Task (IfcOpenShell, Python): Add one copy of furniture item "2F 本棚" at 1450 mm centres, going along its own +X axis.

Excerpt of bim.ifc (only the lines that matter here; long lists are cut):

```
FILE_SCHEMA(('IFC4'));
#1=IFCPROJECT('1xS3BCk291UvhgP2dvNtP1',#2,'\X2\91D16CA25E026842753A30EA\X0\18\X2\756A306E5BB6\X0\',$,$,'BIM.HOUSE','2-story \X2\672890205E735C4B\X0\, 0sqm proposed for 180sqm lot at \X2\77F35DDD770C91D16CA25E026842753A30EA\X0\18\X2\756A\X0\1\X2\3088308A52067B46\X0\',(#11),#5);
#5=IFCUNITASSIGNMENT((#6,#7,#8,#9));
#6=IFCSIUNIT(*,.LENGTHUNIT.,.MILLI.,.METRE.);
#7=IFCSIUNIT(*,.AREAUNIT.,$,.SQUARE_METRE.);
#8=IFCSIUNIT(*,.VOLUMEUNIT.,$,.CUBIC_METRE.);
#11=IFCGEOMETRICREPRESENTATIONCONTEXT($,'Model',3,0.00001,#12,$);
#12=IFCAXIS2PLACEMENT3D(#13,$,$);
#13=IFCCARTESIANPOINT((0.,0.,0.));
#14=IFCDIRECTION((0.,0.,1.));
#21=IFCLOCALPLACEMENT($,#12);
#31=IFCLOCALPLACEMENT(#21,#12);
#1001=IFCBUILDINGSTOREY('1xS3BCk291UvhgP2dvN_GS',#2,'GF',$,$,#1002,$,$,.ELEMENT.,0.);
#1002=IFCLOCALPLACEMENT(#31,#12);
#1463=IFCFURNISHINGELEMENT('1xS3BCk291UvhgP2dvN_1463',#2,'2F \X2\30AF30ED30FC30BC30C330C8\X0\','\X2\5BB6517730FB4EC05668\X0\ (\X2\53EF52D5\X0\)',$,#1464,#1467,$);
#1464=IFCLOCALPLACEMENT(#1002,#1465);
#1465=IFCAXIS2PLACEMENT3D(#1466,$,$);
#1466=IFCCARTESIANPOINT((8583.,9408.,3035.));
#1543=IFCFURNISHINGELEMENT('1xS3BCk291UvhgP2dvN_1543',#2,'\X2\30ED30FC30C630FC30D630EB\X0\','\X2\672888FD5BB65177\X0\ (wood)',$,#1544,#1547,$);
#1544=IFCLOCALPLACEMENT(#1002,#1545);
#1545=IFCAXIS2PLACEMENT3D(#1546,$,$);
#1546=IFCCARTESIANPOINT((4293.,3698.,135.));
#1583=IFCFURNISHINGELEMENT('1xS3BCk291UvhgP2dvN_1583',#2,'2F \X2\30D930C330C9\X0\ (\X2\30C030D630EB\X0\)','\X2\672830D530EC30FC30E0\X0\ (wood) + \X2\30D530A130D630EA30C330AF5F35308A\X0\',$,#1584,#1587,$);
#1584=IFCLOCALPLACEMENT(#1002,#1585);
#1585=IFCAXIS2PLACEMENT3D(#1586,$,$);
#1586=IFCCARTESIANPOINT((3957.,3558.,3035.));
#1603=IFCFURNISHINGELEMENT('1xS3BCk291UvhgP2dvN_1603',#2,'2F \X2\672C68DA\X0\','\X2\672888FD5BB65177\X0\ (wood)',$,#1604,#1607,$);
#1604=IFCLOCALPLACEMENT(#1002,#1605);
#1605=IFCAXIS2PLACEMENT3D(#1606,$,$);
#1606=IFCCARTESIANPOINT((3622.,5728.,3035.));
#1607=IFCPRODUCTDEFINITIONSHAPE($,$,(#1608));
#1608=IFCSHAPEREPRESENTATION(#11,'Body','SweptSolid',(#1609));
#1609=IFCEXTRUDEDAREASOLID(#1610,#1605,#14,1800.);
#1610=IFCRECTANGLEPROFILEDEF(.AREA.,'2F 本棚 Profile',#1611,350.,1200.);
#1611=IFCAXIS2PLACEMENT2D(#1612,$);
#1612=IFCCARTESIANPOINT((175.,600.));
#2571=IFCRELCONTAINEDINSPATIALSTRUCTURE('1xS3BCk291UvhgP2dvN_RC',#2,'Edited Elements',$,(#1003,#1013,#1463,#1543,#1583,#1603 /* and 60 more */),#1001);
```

```python
import ifcopenshell
import ifcopenshell.api.geometry
import ifcopenshell.api.root
import ifcopenshell.util.element
import ifcopenshell.util.placement

model = ifcopenshell.open("bim.ifc")


def reuse_history(source, copy):
    """copy_class also copies each property set's owner history, people and application; keep the originals."""
    for rel in copy.IsDefinedBy:
        if rel.is_a("IfcRelDefinesByProperties") and (history := rel.RelatingPropertyDefinition.OwnerHistory):
            rel.RelatingPropertyDefinition.OwnerHistory = source.OwnerHistory
            ifcopenshell.util.element.remove_deep2(model, history)


source = model.by_guid("1xS3BCk291UvhgP2dvN_1603")
base = ifcopenshell.util.placement.get_local_placement(source.ObjectPlacement)
step = base[:3, 0] * 1450.0

for i in range(1, 2):
    copy = ifcopenshell.api.root.copy_class(model, product=source)
    copy.Representation = ifcopenshell.util.element.copy_deep(
        model, source.Representation, exclude=["IfcGeometricRepresentationContext", "IfcRepresentationMap"]
    )
    reuse_history(source, copy)
    matrix = base.copy()
    matrix[:3, 3] += i * step
    print("added at", matrix[:3, 3].round(3) + 0.0)
    ifcopenshell.api.geometry.edit_object_placement(model, product=copy, matrix=matrix, is_si=False)

model.write("bim_rev.ifc")
```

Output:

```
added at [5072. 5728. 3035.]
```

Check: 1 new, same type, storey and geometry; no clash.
